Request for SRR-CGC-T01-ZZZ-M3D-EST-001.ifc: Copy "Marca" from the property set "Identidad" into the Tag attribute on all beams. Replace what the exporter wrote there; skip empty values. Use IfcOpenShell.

First a look at what the model holds.

```python
import ifcopenshell
import ifcopenshell.util.element

model = ifcopenshell.open("SRR-CGC-T01-ZZZ-M3D-EST-001.ifc")
print(model.schema)
beams = model.by_type("IfcBeam")
print(len(beams), "beams")
for e in beams[:8]:
    source = ifcopenshell.util.element.get_pset(e, "Identidad", "Marca")
    target = e.Tag
    print(e.id(), repr(source), repr(target), sep=" | ")
```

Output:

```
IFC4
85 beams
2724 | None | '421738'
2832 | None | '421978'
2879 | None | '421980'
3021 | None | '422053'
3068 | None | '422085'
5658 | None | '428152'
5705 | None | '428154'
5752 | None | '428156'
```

```python
import ifcopenshell
import ifcopenshell.util.element

model = ifcopenshell.open("SRR-CGC-T01-ZZZ-M3D-EST-001.ifc")

count = 0
for e in model.by_type("IfcBeam"):
    value = ifcopenshell.util.element.get_pset(e, "Identidad", "Marca")
    current = e.Tag
    if not value or not value.strip() or current == value:
        continue
    e.Tag = value
    count += 1

print(count, "beams updated")

model.write("SRR-CGC-T01-ZZZ-M3D-EST-001_updated.ifc")
```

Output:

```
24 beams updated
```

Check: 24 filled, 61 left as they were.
